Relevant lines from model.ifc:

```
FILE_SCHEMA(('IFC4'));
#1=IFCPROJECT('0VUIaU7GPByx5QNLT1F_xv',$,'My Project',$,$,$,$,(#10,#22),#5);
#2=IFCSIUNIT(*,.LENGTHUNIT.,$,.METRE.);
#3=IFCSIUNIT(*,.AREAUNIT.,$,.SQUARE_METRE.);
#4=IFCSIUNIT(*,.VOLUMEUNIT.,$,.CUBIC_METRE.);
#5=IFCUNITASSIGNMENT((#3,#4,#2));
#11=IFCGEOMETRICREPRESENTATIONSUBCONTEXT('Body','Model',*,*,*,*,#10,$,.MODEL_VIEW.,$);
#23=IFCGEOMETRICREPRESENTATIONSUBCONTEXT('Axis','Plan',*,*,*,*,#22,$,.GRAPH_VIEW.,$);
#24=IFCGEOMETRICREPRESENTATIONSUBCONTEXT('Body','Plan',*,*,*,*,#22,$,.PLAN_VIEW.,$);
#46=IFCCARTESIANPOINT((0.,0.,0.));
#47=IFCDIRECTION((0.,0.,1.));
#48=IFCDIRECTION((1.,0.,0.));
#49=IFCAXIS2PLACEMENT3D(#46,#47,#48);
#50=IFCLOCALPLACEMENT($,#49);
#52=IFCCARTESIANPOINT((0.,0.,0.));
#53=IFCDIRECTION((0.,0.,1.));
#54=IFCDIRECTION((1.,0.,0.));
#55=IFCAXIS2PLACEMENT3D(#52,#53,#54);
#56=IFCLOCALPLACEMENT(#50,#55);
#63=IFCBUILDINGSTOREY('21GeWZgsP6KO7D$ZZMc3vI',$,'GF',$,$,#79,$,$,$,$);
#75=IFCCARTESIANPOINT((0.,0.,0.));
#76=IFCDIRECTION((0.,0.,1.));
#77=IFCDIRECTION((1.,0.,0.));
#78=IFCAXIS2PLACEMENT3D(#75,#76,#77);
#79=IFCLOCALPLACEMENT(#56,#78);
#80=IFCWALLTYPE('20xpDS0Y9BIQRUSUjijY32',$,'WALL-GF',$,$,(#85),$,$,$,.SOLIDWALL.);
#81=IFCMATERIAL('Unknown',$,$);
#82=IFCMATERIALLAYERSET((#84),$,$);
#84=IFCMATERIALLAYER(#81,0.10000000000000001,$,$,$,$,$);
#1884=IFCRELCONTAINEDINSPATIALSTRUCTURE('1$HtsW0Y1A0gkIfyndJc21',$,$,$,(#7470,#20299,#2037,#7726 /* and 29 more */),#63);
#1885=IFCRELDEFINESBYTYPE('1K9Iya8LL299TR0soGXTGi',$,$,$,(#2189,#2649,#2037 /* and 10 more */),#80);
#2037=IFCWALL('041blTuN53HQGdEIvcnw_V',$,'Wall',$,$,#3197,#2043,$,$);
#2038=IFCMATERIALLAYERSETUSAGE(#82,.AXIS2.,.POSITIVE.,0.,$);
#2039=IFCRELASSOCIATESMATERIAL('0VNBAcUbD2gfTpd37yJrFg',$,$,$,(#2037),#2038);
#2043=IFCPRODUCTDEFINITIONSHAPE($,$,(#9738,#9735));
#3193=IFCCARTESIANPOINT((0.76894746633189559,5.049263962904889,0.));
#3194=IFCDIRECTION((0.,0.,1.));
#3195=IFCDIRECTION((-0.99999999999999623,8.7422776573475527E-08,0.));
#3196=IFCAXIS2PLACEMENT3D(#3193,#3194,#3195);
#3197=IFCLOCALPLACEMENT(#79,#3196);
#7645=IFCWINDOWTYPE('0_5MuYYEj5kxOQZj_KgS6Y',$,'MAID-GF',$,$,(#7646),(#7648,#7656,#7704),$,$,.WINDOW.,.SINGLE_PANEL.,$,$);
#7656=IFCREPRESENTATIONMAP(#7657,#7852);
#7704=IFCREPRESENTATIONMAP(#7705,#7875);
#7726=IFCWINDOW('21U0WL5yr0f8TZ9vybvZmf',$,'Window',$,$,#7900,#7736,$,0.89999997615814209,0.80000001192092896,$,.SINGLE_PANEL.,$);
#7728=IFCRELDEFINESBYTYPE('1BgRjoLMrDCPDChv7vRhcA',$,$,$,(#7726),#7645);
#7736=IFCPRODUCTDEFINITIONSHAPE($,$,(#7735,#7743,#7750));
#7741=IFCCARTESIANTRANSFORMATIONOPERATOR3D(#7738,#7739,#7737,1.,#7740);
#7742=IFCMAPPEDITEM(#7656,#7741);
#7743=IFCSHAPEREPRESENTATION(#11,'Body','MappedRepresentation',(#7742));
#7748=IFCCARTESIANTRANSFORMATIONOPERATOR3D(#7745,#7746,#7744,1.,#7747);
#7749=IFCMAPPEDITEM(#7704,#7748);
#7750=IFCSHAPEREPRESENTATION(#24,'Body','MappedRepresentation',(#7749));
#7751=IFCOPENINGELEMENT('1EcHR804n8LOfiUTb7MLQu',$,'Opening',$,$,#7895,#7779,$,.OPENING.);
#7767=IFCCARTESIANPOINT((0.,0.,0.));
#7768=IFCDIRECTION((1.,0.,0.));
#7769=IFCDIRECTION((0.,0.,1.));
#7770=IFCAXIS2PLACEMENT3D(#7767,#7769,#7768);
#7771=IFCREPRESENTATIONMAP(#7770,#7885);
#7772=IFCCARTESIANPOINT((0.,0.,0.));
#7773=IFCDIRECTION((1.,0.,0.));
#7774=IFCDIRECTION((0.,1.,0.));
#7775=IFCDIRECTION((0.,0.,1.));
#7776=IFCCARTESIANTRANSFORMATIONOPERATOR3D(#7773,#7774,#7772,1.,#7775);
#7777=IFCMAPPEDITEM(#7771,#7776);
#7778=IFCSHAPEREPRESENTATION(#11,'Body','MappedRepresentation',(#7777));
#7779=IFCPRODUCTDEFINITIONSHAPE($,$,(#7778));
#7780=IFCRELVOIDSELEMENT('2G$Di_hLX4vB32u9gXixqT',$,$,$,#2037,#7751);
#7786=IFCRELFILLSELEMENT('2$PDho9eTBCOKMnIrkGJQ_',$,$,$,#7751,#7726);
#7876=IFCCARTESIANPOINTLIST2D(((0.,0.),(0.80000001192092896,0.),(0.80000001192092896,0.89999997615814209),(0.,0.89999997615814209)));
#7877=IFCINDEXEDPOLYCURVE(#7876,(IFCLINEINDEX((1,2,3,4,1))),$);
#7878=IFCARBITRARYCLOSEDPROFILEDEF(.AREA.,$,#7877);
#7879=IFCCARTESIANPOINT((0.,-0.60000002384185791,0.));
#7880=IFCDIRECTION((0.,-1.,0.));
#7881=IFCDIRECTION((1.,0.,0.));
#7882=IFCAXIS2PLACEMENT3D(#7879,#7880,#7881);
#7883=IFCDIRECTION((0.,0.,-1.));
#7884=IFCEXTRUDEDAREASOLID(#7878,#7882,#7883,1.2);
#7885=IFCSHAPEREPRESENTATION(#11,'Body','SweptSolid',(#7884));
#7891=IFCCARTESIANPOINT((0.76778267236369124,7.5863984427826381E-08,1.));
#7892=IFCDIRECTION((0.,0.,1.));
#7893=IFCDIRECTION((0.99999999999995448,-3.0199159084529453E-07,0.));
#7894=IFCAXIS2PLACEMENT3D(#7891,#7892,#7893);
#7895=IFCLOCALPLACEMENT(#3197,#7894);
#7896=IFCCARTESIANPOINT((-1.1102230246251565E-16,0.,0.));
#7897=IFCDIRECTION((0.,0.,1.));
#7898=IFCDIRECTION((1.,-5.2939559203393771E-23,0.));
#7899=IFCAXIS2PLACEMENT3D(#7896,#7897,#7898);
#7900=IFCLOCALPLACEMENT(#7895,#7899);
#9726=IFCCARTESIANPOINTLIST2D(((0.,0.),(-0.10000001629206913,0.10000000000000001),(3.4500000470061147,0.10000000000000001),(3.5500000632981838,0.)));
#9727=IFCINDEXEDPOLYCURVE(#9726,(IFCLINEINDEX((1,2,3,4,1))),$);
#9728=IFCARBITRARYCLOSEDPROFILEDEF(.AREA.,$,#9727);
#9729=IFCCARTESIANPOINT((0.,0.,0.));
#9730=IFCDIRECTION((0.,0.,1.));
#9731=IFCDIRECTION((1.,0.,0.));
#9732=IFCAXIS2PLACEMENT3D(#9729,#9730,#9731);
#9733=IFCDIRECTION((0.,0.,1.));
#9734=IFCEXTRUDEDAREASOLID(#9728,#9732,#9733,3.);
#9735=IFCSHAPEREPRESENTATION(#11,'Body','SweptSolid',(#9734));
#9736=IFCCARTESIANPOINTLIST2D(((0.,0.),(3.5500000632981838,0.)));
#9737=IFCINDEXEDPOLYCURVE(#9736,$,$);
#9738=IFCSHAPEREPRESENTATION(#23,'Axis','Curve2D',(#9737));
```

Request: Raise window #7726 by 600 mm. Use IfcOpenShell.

```python
import numpy as np
import ifcopenshell
import ifcopenshell.api.geometry
import ifcopenshell.util.placement
import ifcopenshell.util.unit

model = ifcopenshell.open("model.ifc")
unit_scale = ifcopenshell.util.unit.calculate_unit_scale(model)

window = model.by_id(7726)
opening = window.FillsVoids[0].RelatingOpeningElement
dz = 0.6 / unit_scale

shift = np.array([0.0, 0.0, dz])
# The window is placed relative to its opening, so it follows when the opening moves.
matrix = ifcopenshell.util.placement.get_local_placement(opening.ObjectPlacement)
matrix[:3, 3] += shift
ifcopenshell.api.geometry.edit_object_placement(
    model, product=opening, matrix=matrix, is_si=False, should_transform_children=True
)

print(f"moved by {dz * unit_scale:+.3f} m")

model.write("model_rev.ifc")
```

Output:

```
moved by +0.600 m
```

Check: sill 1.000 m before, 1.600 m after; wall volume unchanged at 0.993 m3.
